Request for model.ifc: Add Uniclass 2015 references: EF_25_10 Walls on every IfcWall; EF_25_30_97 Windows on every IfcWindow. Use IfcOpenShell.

First a look at what the model holds.

```python
import ifcopenshell

model = ifcopenshell.open("model.ifc")
print(model.schema)
print("classifications:", [c.Name for c in model.by_type("IfcClassification")])
for ifc_class in ("IfcDoor", "IfcRoof", "IfcStair", "IfcWall", "IfcWindow"):
    print(ifc_class, len(model.by_type(ifc_class)))
```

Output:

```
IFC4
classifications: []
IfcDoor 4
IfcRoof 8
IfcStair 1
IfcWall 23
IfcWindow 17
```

```python
import ifcopenshell
import ifcopenshell.api.classification

model = ifcopenshell.open("model.ifc")

system = ifcopenshell.api.classification.add_classification(model, classification="Uniclass 2015")

codes = {
    "IfcWall": ("EF_25_10", "Walls"),
    "IfcWindow": ("EF_25_30_97", "Windows"),
}
for ifc_class, (code, name) in codes.items():
    products = model.by_type(ifc_class)
    ifcopenshell.api.classification.add_reference(
        model, products=products, classification=system, identification=code, name=name
    )
    print(code, len(products))

model.write("model_updated.ifc")
```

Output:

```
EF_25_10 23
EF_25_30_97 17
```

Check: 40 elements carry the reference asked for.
